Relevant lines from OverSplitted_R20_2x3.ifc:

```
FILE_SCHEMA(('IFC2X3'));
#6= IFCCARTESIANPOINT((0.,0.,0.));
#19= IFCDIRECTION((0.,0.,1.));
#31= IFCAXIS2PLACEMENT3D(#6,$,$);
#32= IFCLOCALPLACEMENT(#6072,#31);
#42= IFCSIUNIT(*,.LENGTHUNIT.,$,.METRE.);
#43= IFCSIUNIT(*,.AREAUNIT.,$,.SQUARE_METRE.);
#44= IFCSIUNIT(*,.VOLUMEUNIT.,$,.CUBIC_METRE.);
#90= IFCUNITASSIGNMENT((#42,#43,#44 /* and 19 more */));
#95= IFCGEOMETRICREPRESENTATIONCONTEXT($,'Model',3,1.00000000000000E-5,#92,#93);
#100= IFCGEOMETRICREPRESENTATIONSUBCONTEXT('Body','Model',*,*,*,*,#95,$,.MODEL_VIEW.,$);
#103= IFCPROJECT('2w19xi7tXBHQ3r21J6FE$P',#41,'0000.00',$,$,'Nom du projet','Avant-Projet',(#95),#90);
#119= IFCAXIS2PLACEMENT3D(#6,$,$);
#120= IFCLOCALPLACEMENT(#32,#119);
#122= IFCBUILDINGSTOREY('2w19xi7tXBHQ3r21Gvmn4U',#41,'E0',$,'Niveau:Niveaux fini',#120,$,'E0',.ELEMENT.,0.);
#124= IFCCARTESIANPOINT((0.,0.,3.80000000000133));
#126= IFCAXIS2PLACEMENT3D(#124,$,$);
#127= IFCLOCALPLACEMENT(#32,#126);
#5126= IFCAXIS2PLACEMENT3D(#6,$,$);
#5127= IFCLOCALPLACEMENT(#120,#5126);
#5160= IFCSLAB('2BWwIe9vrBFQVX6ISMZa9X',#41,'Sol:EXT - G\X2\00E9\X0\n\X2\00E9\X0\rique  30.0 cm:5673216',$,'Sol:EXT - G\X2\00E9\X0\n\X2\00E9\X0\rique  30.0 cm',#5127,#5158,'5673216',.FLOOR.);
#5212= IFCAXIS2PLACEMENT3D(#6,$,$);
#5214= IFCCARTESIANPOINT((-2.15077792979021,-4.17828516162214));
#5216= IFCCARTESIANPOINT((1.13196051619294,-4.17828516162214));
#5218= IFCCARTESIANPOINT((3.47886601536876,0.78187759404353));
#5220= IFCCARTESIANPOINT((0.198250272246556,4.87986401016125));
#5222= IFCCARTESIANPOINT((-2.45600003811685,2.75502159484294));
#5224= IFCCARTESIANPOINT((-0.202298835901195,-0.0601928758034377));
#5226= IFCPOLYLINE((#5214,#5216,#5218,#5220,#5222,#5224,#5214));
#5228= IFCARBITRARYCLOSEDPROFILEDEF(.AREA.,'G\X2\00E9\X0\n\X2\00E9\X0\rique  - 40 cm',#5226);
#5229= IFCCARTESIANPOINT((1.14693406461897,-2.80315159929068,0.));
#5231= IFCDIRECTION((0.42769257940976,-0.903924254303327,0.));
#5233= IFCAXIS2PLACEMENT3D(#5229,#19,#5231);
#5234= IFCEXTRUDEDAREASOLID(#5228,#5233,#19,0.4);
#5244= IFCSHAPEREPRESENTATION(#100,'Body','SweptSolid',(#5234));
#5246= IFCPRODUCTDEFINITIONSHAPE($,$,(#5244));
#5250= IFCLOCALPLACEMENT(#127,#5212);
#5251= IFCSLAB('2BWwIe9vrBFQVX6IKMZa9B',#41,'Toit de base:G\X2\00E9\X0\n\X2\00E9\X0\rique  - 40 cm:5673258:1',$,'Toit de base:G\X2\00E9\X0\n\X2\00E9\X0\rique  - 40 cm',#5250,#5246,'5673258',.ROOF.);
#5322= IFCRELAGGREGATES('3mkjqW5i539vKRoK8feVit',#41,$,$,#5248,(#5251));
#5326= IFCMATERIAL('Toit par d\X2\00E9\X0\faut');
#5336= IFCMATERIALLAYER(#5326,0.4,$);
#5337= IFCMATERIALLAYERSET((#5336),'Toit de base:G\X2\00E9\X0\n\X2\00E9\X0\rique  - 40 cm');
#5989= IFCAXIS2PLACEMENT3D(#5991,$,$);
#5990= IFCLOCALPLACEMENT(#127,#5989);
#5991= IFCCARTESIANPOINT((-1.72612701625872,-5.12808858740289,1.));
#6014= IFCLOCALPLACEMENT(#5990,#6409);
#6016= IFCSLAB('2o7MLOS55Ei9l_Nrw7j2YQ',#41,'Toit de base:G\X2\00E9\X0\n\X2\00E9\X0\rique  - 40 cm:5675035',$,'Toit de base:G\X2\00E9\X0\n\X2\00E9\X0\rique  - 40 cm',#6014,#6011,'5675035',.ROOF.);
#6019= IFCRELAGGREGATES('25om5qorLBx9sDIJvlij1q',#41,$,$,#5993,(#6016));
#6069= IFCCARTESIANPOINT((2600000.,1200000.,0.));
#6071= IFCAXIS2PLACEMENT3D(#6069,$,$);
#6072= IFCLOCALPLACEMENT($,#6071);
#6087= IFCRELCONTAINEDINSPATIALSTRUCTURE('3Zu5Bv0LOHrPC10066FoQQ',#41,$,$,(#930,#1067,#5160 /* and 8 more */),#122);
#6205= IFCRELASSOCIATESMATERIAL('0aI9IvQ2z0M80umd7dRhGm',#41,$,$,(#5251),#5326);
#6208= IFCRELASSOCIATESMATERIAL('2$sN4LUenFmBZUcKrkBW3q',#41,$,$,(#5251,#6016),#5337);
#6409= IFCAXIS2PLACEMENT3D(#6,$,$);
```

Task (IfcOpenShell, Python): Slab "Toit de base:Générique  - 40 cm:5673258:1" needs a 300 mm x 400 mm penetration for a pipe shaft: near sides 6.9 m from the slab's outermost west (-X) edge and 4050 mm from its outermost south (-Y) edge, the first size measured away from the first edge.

```python
import numpy as np
import ifcopenshell
import ifcopenshell.api.feature
import ifcopenshell.api.geometry
import ifcopenshell.api.root
import ifcopenshell.geom
import ifcopenshell.util.placement
import ifcopenshell.util.representation
import ifcopenshell.util.shape
import ifcopenshell.util.unit

model = ifcopenshell.open("OverSplitted_R20_2x3.ifc")
unit_scale = ifcopenshell.util.unit.calculate_unit_scale(model)
settings = ifcopenshell.geom.settings()


def volume(element):
    """Net volume in cubic metres, openings subtracted."""
    shape = ifcopenshell.geom.create_shape(settings, element)
    return ifcopenshell.util.shape.get_volume(shape.geometry)


slab = model.by_guid("2BWwIe9vrBFQVX6IKMZa9B")
before = volume(slab)

# Extent in the slab's own axes, in metres. The edges named are its -X and -Y sides.
slab_shape = ifcopenshell.geom.create_shape(settings, slab)
vertices = ifcopenshell.util.shape.get_vertices(slab_shape.geometry)
x_min, y_min, bottom = vertices.min(axis=0)
top = vertices[:, 2].max()

opening = ifcopenshell.api.root.create_entity(model, ifc_class="IfcOpeningElement", name="Pipe shaft opening")
context = ifcopenshell.util.representation.get_context(model, "Model", "Body", "MODEL_VIEW")
width, depth = 0.3, 0.4
outline = [(0.0, 0.0), (width, 0.0), (width, depth), (0.0, depth), (0.0, 0.0)]
# Overshoot both faces by 50 mm so the cut is clean.
shape = ifcopenshell.api.geometry.add_slab_representation(
    model, context=context, depth=top - bottom + 0.1, polyline=outline
)
ifcopenshell.api.geometry.assign_representation(model, product=opening, representation=shape)

matrix = ifcopenshell.util.placement.get_local_placement(slab.ObjectPlacement)
matrix[:, 3] = matrix @ np.append(np.array([x_min + 6.9, y_min + 4.05, bottom - 0.05]) / unit_scale, 1.0)
ifcopenshell.api.geometry.edit_object_placement(model, product=opening, matrix=matrix, is_si=False)
ifcopenshell.api.feature.add_feature(model, feature=opening, element=slab)

after = volume(slab)

print(f"slab volume {before:.3f} -> {after:.3f} m3")

model.write("OverSplitted_R20_2x3_v2.ifc")
```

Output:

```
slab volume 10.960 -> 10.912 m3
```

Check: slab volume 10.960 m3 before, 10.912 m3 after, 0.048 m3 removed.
